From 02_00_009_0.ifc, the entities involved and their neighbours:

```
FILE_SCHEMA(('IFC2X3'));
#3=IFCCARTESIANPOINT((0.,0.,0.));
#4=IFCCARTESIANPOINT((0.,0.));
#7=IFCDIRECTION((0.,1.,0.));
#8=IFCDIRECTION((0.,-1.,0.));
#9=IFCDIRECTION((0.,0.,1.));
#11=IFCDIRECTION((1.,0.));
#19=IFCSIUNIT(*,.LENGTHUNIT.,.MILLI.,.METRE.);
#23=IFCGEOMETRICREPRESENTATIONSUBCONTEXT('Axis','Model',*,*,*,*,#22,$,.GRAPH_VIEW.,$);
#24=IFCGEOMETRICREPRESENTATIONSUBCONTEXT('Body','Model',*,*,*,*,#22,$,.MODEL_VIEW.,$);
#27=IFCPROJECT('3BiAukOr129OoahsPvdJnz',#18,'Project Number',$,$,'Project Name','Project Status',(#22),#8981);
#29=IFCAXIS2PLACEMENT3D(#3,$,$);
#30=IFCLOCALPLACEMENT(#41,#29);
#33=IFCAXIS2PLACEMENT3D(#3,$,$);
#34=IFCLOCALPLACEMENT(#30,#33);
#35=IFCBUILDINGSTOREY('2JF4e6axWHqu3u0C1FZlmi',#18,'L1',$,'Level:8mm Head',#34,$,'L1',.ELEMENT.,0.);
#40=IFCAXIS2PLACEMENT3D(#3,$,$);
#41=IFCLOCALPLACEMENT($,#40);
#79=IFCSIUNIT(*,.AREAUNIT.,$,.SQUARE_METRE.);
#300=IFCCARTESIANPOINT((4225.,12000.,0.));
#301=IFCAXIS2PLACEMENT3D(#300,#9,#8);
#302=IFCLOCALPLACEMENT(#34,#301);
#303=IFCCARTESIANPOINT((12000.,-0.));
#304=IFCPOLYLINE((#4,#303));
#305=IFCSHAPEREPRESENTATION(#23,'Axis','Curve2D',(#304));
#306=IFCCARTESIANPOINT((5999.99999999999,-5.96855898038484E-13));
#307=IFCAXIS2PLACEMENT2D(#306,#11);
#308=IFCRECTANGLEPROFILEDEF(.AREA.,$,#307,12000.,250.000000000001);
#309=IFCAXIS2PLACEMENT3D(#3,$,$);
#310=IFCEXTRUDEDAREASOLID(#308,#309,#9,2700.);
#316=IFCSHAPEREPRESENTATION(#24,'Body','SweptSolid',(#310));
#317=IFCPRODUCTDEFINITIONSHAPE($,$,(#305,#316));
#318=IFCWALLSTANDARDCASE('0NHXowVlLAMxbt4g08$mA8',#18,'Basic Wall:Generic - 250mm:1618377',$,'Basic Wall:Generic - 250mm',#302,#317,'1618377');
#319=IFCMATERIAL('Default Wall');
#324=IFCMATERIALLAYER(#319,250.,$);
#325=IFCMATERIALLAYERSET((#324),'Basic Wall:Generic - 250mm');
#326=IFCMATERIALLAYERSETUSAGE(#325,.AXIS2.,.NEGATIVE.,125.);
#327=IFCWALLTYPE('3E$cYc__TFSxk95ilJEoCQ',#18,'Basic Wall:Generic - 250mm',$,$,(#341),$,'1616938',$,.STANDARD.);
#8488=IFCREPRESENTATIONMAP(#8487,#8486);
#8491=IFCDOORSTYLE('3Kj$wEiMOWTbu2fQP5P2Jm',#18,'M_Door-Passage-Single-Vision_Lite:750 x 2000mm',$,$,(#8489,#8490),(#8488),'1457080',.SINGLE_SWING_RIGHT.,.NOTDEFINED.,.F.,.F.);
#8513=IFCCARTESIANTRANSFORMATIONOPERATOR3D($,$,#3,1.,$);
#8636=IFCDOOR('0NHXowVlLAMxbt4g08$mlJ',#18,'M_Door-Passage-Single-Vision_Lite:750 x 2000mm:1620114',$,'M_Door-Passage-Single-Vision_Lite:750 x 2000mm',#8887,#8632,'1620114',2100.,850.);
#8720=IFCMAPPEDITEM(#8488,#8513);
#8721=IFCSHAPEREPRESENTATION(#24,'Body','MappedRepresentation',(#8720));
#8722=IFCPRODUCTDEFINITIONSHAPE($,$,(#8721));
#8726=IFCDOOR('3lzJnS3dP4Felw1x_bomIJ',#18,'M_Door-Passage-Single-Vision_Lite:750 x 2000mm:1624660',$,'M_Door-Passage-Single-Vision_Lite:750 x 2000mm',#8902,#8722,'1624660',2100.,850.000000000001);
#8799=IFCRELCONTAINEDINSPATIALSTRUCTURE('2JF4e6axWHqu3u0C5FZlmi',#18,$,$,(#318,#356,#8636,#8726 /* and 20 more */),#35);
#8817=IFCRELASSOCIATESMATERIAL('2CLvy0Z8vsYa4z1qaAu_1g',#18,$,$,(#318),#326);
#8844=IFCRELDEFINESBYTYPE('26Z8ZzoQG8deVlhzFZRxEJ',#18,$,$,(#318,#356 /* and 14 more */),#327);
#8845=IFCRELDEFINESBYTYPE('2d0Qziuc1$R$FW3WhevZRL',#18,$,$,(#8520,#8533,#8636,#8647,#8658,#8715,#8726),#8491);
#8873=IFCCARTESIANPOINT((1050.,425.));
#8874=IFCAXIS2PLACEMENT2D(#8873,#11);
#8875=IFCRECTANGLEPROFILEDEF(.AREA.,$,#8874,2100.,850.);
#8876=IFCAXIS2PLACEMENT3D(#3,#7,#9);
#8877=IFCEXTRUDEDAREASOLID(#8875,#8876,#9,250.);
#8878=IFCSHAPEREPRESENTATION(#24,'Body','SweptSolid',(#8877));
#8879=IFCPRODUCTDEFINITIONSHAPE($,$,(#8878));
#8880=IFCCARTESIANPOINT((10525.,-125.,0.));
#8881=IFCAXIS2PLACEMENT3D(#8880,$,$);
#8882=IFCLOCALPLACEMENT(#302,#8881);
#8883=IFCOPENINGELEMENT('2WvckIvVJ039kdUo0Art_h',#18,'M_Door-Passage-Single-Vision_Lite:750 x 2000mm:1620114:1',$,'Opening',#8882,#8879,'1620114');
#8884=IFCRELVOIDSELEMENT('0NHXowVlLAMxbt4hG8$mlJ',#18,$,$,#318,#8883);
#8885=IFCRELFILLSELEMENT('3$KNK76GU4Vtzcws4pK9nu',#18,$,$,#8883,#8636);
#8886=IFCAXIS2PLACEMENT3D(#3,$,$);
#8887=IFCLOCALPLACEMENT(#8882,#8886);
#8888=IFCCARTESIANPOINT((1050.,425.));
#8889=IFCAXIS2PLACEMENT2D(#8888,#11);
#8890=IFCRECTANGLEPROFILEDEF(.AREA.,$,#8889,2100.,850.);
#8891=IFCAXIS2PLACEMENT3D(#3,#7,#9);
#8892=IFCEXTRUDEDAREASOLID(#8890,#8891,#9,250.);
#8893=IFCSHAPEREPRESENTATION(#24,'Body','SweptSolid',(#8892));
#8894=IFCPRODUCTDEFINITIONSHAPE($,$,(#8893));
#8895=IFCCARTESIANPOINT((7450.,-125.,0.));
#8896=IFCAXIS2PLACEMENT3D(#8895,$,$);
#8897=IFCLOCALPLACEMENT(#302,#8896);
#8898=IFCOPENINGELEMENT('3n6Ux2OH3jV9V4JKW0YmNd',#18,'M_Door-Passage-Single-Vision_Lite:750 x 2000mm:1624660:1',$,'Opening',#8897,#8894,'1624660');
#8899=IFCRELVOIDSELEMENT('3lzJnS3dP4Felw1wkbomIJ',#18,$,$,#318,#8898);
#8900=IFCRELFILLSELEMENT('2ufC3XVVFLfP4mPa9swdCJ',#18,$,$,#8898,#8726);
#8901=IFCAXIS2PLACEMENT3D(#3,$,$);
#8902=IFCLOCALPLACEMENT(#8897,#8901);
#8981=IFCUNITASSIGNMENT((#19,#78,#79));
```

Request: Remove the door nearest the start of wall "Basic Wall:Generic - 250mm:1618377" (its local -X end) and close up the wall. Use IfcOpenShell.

```python
import ifcopenshell
import ifcopenshell.api.feature
import ifcopenshell.api.root
import ifcopenshell.geom
import ifcopenshell.util.shape

model = ifcopenshell.open("02_00_009_0.ifc")
settings = ifcopenshell.geom.settings()


def volume(element):
    """Net volume in cubic metres, openings subtracted."""
    shape = ifcopenshell.geom.create_shape(settings, element)
    return ifcopenshell.util.shape.get_volume(shape.geometry)


door = model.by_guid("3lzJnS3dP4Felw1x_bomIJ")
opening = door.FillsVoids[0].RelatingOpeningElement
wall = opening.VoidsElements[0].RelatingBuildingElement
before = volume(wall)

ifcopenshell.api.root.remove_product(model, product=door)
ifcopenshell.api.feature.remove_feature(model, feature=opening)

after = volume(wall)

print(f"wall volume {before:.3f} -> {after:.3f} m3")

model.write("02_00_009_0_v2.ifc")
```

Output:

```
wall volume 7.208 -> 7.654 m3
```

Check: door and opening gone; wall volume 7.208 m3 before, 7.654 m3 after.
